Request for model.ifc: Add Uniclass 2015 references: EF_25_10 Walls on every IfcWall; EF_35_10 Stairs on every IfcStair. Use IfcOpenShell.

First a look at what the model holds.

```python
import ifcopenshell

model = ifcopenshell.open("model.ifc")
print(model.schema)
print("classifications:", [c.Name for c in model.by_type("IfcClassification")])
for ifc_class in ("IfcDoor", "IfcRoof", "IfcStair", "IfcWall", "IfcWindow"):
    print(ifc_class, len(model.by_type(ifc_class)))
```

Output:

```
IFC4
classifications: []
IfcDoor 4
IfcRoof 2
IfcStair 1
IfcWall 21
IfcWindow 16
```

```python
import ifcopenshell
import ifcopenshell.api.classification

model = ifcopenshell.open("model.ifc")

system = ifcopenshell.api.classification.add_classification(model, classification="Uniclass 2015")

codes = {
    "IfcWall": ("EF_25_10", "Walls"),
    "IfcStair": ("EF_35_10", "Stairs"),
}
for ifc_class, (code, name) in codes.items():
    products = model.by_type(ifc_class)
    ifcopenshell.api.classification.add_reference(
        model, products=products, classification=system, identification=code, name=name
    )
    print(code, len(products))

model.write("model_rev.ifc")
```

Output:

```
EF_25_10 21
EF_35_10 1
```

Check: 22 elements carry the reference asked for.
